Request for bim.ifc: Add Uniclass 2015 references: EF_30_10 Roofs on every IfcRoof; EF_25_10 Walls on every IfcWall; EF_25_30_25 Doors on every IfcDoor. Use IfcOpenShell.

First a look at what the model holds.

```python
import ifcopenshell

model = ifcopenshell.open("bim.ifc")
print(model.schema)
print("classifications:", [c.Name for c in model.by_type("IfcClassification")])
for ifc_class in ("IfcDoor", "IfcRoof", "IfcStair", "IfcWall", "IfcWindow"):
    print(ifc_class, len(model.by_type(ifc_class)))
```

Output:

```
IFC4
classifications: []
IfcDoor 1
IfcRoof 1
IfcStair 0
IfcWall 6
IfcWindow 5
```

```python
import ifcopenshell
import ifcopenshell.api.classification

model = ifcopenshell.open("bim.ifc")

system = ifcopenshell.api.classification.add_classification(model, classification="Uniclass 2015")

codes = {
    "IfcRoof": ("EF_30_10", "Roofs"),
    "IfcWall": ("EF_25_10", "Walls"),
    "IfcDoor": ("EF_25_30_25", "Doors"),
}
for ifc_class, (code, name) in codes.items():
    products = model.by_type(ifc_class)
    ifcopenshell.api.classification.add_reference(
        model, products=products, classification=system, identification=code, name=name
    )
    print(code, len(products))

model.write("bim_updated.ifc")
```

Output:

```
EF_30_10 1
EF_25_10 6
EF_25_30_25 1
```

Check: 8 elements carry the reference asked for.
